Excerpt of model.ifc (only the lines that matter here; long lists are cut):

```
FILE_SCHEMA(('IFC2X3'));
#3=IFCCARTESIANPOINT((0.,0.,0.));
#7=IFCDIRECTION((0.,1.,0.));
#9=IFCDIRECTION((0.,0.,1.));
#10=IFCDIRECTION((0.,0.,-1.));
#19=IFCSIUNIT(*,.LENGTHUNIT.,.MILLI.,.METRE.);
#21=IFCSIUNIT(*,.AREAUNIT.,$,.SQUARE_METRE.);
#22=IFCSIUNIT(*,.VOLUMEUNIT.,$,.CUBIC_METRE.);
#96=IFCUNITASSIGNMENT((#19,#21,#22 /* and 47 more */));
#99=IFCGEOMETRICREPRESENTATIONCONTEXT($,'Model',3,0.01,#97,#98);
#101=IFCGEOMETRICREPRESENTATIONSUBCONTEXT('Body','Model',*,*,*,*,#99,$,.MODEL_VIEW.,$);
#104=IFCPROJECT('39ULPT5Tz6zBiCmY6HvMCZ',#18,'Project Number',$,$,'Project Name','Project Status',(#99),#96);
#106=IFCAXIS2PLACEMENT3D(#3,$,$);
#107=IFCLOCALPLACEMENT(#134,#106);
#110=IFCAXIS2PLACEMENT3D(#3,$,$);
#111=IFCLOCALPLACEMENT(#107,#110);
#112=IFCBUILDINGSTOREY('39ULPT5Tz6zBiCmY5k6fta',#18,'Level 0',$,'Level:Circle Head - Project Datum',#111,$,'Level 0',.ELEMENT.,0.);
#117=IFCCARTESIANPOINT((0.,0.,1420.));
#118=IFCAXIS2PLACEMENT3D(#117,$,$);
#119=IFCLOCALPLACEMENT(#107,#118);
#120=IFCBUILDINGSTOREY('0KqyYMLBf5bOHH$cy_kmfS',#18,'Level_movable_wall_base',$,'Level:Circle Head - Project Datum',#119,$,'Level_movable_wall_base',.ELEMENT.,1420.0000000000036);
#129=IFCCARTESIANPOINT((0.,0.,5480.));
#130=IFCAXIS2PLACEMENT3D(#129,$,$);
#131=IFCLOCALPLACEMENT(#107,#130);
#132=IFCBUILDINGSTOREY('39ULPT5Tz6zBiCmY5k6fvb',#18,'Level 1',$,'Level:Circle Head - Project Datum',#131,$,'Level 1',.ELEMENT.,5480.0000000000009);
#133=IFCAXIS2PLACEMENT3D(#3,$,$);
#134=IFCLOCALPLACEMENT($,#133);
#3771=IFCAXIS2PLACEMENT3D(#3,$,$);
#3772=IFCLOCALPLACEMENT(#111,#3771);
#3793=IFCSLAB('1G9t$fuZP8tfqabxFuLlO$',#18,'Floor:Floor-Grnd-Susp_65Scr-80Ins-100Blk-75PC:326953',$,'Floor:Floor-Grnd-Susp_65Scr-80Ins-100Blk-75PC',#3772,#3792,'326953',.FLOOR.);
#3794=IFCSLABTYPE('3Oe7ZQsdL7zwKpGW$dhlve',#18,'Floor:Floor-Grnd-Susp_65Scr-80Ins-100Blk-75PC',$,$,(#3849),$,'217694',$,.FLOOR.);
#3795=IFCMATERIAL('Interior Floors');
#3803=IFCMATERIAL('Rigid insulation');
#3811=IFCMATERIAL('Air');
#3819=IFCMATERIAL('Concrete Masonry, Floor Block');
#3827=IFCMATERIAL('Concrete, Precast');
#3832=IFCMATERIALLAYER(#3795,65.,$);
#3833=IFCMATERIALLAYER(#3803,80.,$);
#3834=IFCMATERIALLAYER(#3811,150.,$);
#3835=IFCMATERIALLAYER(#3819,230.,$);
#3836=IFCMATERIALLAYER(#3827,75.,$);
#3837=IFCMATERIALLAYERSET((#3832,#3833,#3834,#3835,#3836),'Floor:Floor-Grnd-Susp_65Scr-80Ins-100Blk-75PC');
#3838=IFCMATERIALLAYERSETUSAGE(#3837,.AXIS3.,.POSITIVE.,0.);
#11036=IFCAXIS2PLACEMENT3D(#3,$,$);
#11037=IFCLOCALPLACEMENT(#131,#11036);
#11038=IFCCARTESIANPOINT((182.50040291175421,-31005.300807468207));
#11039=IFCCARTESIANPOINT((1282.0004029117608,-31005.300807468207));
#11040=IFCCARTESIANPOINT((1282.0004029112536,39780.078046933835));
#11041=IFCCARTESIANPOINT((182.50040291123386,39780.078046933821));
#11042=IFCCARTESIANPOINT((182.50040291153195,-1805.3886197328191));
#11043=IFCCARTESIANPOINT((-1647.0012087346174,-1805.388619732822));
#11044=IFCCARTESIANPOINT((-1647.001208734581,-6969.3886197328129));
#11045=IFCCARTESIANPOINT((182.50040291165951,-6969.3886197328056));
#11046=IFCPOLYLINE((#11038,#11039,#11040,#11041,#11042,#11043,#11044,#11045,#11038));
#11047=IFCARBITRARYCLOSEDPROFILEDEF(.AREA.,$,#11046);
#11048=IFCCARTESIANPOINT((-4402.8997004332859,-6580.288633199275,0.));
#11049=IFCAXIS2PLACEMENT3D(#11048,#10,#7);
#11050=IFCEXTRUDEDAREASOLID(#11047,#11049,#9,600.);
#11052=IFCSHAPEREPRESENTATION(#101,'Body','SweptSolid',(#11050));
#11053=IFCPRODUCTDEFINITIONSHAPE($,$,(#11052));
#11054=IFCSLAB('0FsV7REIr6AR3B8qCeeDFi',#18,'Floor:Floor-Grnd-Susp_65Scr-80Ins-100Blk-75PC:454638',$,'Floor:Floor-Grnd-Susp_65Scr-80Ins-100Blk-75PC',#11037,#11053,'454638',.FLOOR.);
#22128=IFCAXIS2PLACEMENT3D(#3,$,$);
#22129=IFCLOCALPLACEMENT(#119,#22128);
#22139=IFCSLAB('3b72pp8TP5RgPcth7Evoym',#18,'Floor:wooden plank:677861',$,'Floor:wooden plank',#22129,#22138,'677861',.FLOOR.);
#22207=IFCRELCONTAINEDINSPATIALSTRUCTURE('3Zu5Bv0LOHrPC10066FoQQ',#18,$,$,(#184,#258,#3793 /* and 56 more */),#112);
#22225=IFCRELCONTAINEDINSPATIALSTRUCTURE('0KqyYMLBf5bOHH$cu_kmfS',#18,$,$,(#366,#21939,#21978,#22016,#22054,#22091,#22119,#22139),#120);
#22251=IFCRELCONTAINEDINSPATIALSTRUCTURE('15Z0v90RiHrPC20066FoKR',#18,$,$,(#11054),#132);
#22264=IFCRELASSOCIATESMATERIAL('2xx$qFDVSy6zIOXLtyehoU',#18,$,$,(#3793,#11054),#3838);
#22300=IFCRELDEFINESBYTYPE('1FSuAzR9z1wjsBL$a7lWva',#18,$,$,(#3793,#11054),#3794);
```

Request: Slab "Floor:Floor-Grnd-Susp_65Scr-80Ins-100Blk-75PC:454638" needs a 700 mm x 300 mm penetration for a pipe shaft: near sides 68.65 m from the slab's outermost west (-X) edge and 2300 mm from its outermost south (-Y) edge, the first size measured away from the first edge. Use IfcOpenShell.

```python
import numpy as np
import ifcopenshell
import ifcopenshell.api.feature
import ifcopenshell.api.geometry
import ifcopenshell.api.root
import ifcopenshell.geom
import ifcopenshell.util.placement
import ifcopenshell.util.representation
import ifcopenshell.util.shape
import ifcopenshell.util.unit

model = ifcopenshell.open("model.ifc")
unit_scale = ifcopenshell.util.unit.calculate_unit_scale(model)
settings = ifcopenshell.geom.settings()


def volume(element):
    """Net volume in cubic metres, openings subtracted."""
    shape = ifcopenshell.geom.create_shape(settings, element)
    return ifcopenshell.util.shape.get_volume(shape.geometry)


slab = model.by_guid("0FsV7REIr6AR3B8qCeeDFi")
before = volume(slab)

# Extent in the slab's own axes, in metres. The edges named are its -X and -Y sides.
slab_shape = ifcopenshell.geom.create_shape(settings, slab)
vertices = ifcopenshell.util.shape.get_vertices(slab_shape.geometry)
x_min, y_min, bottom = vertices.min(axis=0)
top = vertices[:, 2].max()

opening = ifcopenshell.api.root.create_entity(model, ifc_class="IfcOpeningElement", name="Pipe shaft opening")
context = ifcopenshell.util.representation.get_context(model, "Model", "Body", "MODEL_VIEW")
width, depth = 0.7, 0.3
outline = [(0.0, 0.0), (width, 0.0), (width, depth), (0.0, depth), (0.0, 0.0)]
# Overshoot both faces by 50 mm so the cut is clean.
shape = ifcopenshell.api.geometry.add_slab_representation(
    model, context=context, depth=top - bottom + 0.1, polyline=outline
)
ifcopenshell.api.geometry.assign_representation(model, product=opening, representation=shape)

matrix = ifcopenshell.util.placement.get_local_placement(slab.ObjectPlacement)
matrix[:, 3] = matrix @ np.append(np.array([x_min + 68.65, y_min + 2.3, bottom - 0.05]) / unit_scale, 1.0)
ifcopenshell.api.geometry.edit_object_placement(model, product=opening, matrix=matrix, is_si=False)
ifcopenshell.api.feature.add_feature(model, feature=opening, element=slab)

after = volume(slab)

print(f"slab volume {before:.3f} -> {after:.3f} m3")

model.write("model_edited.ifc")
```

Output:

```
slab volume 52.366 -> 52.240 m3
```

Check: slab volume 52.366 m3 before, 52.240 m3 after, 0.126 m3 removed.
